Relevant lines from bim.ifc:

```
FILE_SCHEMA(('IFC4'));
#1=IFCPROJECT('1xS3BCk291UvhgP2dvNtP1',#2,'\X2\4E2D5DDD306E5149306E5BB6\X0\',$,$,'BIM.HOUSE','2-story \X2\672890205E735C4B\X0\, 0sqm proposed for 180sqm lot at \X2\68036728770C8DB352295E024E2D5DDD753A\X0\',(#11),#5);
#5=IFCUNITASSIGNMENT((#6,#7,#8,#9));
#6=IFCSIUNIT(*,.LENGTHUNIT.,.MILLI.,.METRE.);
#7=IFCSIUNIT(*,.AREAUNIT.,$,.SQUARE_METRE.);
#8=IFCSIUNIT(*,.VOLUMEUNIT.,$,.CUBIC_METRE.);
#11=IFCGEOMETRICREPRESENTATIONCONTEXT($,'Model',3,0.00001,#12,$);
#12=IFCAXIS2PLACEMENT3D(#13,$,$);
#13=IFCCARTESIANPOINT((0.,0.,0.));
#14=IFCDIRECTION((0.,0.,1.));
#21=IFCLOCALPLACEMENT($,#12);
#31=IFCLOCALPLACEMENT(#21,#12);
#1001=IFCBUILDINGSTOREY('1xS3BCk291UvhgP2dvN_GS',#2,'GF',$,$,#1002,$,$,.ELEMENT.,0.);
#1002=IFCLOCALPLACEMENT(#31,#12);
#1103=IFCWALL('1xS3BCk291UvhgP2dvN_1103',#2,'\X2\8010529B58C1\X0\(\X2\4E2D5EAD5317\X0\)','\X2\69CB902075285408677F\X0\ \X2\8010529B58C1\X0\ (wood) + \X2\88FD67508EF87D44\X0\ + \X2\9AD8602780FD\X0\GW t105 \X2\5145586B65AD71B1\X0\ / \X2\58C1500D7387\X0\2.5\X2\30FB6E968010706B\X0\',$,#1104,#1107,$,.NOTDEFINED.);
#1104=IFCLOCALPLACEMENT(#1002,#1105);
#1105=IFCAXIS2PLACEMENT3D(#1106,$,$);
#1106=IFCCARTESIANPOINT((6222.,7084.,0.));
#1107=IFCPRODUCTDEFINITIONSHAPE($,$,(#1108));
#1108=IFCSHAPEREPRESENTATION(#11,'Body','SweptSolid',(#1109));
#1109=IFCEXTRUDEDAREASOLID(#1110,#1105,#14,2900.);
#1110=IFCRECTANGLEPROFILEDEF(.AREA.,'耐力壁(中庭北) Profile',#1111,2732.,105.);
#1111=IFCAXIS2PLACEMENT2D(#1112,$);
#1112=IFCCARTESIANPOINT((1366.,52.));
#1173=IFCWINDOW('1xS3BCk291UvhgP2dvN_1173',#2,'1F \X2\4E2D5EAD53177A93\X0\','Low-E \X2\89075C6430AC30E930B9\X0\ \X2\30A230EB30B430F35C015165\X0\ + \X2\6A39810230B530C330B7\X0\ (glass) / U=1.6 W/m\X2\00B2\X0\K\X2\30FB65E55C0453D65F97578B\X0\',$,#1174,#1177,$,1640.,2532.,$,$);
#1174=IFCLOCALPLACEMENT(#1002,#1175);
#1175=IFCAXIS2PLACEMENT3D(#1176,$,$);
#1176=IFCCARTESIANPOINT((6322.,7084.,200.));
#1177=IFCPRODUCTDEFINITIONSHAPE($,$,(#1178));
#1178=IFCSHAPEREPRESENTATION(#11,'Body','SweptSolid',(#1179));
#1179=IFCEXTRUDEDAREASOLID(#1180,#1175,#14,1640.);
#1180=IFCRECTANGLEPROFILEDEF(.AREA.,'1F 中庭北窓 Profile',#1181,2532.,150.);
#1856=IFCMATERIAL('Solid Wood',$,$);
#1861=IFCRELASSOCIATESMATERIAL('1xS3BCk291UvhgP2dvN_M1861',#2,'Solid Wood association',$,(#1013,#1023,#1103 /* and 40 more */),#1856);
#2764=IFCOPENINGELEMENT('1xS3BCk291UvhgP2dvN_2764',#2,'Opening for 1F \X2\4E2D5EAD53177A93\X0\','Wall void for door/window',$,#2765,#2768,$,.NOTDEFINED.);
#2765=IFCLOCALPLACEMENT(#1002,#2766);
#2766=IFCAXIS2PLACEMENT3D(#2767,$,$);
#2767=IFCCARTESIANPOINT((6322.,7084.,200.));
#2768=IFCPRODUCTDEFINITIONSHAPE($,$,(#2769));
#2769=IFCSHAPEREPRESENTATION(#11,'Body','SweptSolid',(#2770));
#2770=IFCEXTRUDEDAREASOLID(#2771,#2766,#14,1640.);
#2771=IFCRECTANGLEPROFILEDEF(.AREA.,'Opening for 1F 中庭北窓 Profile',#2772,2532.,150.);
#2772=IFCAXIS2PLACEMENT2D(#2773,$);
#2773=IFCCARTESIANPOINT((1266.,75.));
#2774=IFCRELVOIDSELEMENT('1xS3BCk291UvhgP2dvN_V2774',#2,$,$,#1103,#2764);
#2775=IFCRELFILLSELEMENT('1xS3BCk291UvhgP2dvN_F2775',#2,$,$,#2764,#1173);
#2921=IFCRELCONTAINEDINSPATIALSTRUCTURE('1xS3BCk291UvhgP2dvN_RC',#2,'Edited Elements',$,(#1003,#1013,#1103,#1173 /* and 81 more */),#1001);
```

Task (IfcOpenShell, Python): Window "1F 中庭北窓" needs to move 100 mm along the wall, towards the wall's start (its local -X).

```python
import ifcopenshell
import ifcopenshell.api.geometry
import ifcopenshell.util.placement
import ifcopenshell.util.unit

model = ifcopenshell.open("bim.ifc")
unit_scale = ifcopenshell.util.unit.calculate_unit_scale(model)

window = model.by_guid("1xS3BCk291UvhgP2dvN_1173")
opening = window.FillsVoids[0].RelatingOpeningElement
wall = opening.VoidsElements[0].RelatingBuildingElement

wall_matrix = ifcopenshell.util.placement.get_local_placement(wall.ObjectPlacement)
shift = wall_matrix[:3, 0] * -0.1 / unit_scale
before = ifcopenshell.util.placement.get_local_placement(window.ObjectPlacement)[:3, 3].copy()

# The window is not placed relative to its opening, so move both.
for product in (opening, window):
    matrix = ifcopenshell.util.placement.get_local_placement(product.ObjectPlacement)
    matrix[:3, 3] += shift
    ifcopenshell.api.geometry.edit_object_placement(model, product=product, matrix=matrix, is_si=False)

after = ifcopenshell.util.placement.get_local_placement(window.ObjectPlacement)[:3, 3]
print("window moved by", (after - before).round(3) + 0.0)

model.write("bim-out.ifc")
```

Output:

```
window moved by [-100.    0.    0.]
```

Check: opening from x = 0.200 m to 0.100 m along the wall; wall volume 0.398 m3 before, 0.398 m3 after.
